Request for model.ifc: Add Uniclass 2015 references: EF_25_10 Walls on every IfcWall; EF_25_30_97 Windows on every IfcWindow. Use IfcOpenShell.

First a look at what the model holds.

```python
import ifcopenshell

model = ifcopenshell.open("model.ifc")
print(model.schema)
print("classifications:", [c.Name for c in model.by_type("IfcClassification")])
for ifc_class in ("IfcDoor", "IfcRoof", "IfcStair", "IfcWall", "IfcWindow"):
    print(ifc_class, len(model.by_type(ifc_class)))
```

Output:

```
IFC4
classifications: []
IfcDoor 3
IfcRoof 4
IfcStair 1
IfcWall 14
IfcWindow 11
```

```python
import ifcopenshell
import ifcopenshell.api.classification

model = ifcopenshell.open("model.ifc")

system = ifcopenshell.api.classification.add_classification(model, classification="Uniclass 2015")

codes = {
    "IfcWall": ("EF_25_10", "Walls"),
    "IfcWindow": ("EF_25_30_97", "Windows"),
}
for ifc_class, (code, name) in codes.items():
    products = model.by_type(ifc_class)
    ifcopenshell.api.classification.add_reference(
        model, products=products, classification=system, identification=code, name=name
    )
    print(code, len(products))

model.write("model_v2.ifc")
```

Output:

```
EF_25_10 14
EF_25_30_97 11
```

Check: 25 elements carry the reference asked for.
